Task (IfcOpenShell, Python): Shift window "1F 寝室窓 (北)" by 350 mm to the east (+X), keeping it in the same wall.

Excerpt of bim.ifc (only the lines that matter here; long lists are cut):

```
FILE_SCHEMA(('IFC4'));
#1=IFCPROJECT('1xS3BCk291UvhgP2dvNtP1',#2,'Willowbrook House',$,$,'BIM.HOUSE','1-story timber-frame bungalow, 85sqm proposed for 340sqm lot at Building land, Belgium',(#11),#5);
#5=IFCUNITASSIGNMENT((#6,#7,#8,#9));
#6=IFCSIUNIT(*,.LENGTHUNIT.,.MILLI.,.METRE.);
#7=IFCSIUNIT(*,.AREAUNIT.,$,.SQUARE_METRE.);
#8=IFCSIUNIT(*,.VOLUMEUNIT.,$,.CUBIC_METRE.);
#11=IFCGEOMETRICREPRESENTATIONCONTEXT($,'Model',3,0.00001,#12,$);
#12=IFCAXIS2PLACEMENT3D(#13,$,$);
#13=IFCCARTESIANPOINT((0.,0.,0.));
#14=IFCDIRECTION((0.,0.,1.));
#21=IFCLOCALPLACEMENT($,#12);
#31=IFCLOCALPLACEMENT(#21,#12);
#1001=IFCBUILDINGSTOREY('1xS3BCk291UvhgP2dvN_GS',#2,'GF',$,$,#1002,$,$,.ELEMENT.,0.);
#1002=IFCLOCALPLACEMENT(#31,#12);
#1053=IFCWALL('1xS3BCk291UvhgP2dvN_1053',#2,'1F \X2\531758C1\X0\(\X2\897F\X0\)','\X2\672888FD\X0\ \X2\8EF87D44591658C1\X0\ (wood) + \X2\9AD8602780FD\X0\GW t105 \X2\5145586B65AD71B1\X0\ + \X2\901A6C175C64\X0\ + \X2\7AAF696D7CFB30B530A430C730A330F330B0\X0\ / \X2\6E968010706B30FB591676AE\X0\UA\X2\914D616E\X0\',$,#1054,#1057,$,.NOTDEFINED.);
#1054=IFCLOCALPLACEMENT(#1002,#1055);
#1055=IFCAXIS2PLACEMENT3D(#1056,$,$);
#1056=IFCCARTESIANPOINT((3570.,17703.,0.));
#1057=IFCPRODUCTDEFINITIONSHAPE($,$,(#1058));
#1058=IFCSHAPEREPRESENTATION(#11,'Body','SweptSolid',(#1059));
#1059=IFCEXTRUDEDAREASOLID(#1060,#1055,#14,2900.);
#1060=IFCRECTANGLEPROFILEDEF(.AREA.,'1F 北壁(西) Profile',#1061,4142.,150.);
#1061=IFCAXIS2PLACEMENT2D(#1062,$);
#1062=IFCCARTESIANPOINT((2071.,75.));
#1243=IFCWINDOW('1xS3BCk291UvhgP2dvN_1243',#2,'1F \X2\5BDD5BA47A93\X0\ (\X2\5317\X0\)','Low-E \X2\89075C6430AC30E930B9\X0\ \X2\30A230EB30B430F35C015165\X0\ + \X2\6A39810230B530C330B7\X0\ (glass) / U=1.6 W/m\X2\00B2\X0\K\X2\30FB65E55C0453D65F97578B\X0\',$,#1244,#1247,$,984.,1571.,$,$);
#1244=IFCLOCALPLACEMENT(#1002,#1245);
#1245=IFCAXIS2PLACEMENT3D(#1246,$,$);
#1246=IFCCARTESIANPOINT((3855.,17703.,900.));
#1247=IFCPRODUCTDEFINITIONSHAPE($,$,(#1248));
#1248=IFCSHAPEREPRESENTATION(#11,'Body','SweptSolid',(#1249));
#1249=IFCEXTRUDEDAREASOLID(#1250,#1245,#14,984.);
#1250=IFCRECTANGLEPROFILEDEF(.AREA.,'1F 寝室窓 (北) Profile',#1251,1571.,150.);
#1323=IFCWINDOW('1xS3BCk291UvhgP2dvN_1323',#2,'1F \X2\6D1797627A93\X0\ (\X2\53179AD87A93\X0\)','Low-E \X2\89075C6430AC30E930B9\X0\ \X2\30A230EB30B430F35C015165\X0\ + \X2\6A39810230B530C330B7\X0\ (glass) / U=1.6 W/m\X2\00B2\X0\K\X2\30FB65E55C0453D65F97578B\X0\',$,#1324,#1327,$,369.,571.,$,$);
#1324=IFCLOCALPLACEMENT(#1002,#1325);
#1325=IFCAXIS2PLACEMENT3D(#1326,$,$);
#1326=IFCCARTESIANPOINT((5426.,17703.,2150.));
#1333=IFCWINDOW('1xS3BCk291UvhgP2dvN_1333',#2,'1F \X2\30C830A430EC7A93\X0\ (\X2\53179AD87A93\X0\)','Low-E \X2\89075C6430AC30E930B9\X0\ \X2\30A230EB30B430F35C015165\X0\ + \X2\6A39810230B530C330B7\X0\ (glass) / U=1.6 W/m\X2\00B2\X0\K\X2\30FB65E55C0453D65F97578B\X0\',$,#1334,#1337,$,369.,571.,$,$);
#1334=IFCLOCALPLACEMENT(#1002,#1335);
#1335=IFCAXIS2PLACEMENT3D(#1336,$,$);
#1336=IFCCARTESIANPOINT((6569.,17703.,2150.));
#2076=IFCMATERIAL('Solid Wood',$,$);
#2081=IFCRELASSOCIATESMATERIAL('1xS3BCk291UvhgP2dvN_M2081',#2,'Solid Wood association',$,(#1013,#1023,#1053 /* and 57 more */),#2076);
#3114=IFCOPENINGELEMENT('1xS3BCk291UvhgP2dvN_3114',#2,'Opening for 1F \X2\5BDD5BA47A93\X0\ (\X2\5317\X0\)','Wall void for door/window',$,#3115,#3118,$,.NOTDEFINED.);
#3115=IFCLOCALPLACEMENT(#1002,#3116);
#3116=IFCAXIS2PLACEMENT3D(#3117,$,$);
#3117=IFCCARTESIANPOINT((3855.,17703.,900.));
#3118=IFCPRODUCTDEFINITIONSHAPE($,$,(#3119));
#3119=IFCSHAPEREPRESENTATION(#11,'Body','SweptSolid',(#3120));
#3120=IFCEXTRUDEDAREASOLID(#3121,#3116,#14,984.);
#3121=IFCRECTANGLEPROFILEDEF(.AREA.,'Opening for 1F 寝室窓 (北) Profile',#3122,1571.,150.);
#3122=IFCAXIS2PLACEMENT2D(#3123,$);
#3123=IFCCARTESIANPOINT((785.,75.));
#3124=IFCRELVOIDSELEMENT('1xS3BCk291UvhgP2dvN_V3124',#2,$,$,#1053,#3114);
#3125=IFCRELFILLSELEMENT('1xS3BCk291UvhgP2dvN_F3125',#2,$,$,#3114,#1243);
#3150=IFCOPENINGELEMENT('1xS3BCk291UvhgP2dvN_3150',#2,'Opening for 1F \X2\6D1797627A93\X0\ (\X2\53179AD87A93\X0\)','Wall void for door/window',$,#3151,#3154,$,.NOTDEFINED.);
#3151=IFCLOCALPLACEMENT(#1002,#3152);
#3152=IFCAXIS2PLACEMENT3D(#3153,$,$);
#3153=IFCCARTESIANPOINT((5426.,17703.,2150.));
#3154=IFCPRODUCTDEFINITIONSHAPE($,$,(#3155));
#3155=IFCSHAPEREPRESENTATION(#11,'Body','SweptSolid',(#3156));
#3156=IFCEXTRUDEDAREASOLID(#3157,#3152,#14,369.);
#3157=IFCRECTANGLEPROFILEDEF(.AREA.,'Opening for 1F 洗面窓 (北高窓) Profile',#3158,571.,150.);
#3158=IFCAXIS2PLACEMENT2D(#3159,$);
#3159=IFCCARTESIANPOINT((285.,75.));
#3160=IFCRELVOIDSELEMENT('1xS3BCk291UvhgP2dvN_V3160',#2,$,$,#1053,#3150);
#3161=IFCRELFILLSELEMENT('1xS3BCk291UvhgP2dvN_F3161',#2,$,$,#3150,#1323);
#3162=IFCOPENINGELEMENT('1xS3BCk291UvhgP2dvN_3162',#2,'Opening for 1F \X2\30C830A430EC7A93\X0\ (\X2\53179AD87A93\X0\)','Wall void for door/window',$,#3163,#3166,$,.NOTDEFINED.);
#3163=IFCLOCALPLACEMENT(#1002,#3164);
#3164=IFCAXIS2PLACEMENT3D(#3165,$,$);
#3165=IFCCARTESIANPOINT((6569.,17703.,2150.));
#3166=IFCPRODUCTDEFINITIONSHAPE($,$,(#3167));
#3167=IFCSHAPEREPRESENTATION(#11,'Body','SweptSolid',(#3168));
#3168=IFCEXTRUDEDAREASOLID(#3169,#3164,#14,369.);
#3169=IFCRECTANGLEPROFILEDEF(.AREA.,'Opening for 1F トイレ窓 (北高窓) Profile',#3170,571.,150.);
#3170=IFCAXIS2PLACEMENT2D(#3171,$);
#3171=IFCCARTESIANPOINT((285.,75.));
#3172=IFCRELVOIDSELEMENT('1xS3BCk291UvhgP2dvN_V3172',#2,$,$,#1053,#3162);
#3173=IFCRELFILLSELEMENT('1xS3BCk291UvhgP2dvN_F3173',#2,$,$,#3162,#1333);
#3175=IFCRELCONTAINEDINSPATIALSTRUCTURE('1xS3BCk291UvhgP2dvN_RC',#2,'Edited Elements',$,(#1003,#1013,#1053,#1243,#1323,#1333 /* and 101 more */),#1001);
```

```python
import ifcopenshell
import ifcopenshell.api.geometry
import ifcopenshell.util.placement
import ifcopenshell.util.unit

model = ifcopenshell.open("bim.ifc")
unit_scale = ifcopenshell.util.unit.calculate_unit_scale(model)

window = model.by_guid("1xS3BCk291UvhgP2dvN_1243")
opening = window.FillsVoids[0].RelatingOpeningElement
wall = opening.VoidsElements[0].RelatingBuildingElement

wall_matrix = ifcopenshell.util.placement.get_local_placement(wall.ObjectPlacement)
shift = wall_matrix[:3, 0] * 0.35 / unit_scale
before = ifcopenshell.util.placement.get_local_placement(window.ObjectPlacement)[:3, 3].copy()

# The window is not placed relative to its opening, so move both.
for product in (opening, window):
    matrix = ifcopenshell.util.placement.get_local_placement(product.ObjectPlacement)
    matrix[:3, 3] += shift
    ifcopenshell.api.geometry.edit_object_placement(model, product=product, matrix=matrix, is_si=False)

after = ifcopenshell.util.placement.get_local_placement(window.ObjectPlacement)[:3, 3]
print("window moved by", (after - before).round(3) + 0.0)

model.write("bim_edited.ifc")
```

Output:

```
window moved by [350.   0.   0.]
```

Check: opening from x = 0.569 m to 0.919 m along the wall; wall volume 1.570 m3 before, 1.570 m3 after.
